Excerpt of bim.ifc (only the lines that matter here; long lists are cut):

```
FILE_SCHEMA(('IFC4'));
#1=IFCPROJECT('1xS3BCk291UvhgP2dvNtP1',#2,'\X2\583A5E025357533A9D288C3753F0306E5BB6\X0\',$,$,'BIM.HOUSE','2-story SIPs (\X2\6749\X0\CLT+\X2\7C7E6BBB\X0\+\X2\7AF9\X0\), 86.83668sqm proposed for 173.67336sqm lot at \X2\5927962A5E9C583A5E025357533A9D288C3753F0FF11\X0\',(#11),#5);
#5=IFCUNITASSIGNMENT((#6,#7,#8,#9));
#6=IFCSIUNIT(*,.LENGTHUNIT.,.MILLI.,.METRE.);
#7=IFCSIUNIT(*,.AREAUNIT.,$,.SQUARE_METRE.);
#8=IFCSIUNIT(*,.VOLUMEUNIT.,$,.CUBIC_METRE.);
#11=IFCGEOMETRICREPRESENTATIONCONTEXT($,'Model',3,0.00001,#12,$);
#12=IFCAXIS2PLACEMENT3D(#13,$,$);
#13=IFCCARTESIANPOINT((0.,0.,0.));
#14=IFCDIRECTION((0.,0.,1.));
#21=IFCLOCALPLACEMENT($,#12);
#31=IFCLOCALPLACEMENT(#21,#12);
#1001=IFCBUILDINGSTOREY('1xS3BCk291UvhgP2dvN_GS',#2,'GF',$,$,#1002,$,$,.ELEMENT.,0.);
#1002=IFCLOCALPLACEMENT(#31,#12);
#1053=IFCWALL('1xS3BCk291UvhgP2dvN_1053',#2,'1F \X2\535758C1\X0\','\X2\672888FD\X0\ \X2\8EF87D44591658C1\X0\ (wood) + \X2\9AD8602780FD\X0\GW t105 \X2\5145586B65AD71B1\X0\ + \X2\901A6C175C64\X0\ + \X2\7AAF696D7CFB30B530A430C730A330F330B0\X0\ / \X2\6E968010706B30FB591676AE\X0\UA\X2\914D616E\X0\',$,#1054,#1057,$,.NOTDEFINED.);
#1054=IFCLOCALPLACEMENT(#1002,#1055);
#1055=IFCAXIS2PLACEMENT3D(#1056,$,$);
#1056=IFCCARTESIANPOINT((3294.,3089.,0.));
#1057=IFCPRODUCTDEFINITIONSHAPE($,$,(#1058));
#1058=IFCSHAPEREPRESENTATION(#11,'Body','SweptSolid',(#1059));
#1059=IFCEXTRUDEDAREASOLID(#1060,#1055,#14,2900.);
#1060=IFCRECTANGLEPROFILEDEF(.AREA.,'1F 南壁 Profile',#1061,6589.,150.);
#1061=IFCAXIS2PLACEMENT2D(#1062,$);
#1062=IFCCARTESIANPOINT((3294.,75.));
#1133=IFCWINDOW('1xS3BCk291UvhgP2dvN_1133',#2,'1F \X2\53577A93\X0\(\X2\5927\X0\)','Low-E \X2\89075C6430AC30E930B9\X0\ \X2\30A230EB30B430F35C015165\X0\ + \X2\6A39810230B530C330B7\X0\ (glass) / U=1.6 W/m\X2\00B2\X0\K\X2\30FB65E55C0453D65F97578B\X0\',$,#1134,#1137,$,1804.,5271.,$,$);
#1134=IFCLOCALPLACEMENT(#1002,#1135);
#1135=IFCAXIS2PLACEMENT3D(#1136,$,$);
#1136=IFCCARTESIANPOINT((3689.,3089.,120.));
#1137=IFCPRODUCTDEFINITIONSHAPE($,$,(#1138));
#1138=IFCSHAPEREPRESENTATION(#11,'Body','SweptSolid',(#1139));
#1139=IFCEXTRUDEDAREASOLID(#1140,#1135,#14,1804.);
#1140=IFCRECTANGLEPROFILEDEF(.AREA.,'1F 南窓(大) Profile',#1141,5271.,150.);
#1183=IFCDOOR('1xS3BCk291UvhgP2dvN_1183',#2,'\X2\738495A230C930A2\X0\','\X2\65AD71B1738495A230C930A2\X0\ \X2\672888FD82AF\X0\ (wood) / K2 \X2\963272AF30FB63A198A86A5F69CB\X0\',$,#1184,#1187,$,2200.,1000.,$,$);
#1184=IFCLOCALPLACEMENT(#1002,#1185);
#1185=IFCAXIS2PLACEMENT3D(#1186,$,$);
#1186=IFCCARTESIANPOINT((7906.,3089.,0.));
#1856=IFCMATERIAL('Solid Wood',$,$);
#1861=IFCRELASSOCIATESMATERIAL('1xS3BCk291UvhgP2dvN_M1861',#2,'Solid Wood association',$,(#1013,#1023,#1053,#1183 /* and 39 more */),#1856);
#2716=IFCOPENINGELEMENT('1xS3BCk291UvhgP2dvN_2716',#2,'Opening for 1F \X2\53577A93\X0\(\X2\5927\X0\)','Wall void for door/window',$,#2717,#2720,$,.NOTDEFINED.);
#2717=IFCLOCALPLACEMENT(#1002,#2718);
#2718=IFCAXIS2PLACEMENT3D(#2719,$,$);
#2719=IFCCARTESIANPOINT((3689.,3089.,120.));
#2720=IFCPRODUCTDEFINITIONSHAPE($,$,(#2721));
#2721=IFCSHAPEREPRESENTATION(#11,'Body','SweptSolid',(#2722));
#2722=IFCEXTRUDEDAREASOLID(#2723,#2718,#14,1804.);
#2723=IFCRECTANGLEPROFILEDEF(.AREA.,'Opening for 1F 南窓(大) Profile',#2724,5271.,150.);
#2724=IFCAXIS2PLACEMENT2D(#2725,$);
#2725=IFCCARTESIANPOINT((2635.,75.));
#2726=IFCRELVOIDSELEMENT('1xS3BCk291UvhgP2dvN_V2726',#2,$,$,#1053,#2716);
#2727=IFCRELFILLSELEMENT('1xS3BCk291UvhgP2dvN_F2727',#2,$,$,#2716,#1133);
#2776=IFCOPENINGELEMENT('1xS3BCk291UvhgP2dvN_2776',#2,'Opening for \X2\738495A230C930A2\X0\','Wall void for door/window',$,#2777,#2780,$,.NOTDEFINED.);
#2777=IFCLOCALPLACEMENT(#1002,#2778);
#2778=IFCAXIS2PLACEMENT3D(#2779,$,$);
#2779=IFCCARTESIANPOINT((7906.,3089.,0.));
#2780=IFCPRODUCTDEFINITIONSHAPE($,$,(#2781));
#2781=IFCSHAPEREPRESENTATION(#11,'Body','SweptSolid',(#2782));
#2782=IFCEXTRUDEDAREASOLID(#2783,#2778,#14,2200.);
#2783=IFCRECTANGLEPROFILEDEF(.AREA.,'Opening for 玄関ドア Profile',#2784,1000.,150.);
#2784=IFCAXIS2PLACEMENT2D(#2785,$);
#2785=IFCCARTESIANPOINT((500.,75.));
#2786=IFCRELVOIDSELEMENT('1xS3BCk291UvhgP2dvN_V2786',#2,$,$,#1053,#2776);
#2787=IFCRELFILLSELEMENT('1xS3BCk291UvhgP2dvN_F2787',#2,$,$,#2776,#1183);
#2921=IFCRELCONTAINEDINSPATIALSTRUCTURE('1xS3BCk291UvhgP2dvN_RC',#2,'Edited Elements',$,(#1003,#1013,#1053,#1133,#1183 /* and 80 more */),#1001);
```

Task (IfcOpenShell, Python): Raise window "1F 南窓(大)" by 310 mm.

```python
import numpy as np
import ifcopenshell
import ifcopenshell.api.geometry
import ifcopenshell.util.placement
import ifcopenshell.util.unit

model = ifcopenshell.open("bim.ifc")
unit_scale = ifcopenshell.util.unit.calculate_unit_scale(model)

window = model.by_guid("1xS3BCk291UvhgP2dvN_1133")
opening = window.FillsVoids[0].RelatingOpeningElement
dz = 0.31 / unit_scale

shift = np.array([0.0, 0.0, dz])
# The window is not placed relative to its opening, so move both.
for product in (opening, window):
    matrix = ifcopenshell.util.placement.get_local_placement(product.ObjectPlacement)
    matrix[:3, 3] += shift
    ifcopenshell.api.geometry.edit_object_placement(model, product=product, matrix=matrix, is_si=False)

print(f"moved by {dz * unit_scale:+.3f} m")

model.write("bim-out.ifc")
```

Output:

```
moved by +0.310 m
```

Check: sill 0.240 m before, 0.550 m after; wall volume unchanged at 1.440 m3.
